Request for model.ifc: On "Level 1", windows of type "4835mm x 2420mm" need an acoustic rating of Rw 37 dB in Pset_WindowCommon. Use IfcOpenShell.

First a look at what the model holds.

```python
import ifcopenshell
import ifcopenshell.util.element

model = ifcopenshell.open("model.ifc")
print(model.schema)
storey = next(s for s in model.by_type("IfcBuildingStorey") if s.Name == "Level 1")
windows = [e for e in ifcopenshell.util.element.get_decomposition(storey) if e.is_a("IfcWindow")]
seen = {}
for e in windows:
    element_type = ifcopenshell.util.element.get_type(e)
    key = (element_type.Name if element_type != e and element_type else None, ifcopenshell.util.element.get_pset(e, "Pset_WindowCommon", "AcousticRating"))
    seen[key] = seen.get(key, 0) + 1
for (name, value), count in sorted(seen.items(), key=str):
    print(count, "x", name, "|", value)
```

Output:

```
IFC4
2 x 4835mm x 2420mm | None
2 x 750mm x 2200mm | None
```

```python
import ifcopenshell
import ifcopenshell.api.pset
import ifcopenshell.util.element

model = ifcopenshell.open("model.ifc")

storey = next(s for s in model.by_type("IfcBuildingStorey") if s.Name == "Level 1")
windows = [e for e in ifcopenshell.util.element.get_decomposition(storey) if e.is_a("IfcWindow")]

count = 0
for e in windows:
    element_type = ifcopenshell.util.element.get_type(e)
    if element_type in (None, e) or element_type.Name != "4835mm x 2420mm":
        continue
    # add_pset returns the element's existing set when there is one.
    pset = ifcopenshell.api.pset.add_pset(model, product=e, name="Pset_WindowCommon")
    ifcopenshell.api.pset.edit_pset(model, pset=pset, properties={"AcousticRating": "Rw 37 dB"})
    count += 1

print(count, "windows updated")

model.write("model-out.ifc")
```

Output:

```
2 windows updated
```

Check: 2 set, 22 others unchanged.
